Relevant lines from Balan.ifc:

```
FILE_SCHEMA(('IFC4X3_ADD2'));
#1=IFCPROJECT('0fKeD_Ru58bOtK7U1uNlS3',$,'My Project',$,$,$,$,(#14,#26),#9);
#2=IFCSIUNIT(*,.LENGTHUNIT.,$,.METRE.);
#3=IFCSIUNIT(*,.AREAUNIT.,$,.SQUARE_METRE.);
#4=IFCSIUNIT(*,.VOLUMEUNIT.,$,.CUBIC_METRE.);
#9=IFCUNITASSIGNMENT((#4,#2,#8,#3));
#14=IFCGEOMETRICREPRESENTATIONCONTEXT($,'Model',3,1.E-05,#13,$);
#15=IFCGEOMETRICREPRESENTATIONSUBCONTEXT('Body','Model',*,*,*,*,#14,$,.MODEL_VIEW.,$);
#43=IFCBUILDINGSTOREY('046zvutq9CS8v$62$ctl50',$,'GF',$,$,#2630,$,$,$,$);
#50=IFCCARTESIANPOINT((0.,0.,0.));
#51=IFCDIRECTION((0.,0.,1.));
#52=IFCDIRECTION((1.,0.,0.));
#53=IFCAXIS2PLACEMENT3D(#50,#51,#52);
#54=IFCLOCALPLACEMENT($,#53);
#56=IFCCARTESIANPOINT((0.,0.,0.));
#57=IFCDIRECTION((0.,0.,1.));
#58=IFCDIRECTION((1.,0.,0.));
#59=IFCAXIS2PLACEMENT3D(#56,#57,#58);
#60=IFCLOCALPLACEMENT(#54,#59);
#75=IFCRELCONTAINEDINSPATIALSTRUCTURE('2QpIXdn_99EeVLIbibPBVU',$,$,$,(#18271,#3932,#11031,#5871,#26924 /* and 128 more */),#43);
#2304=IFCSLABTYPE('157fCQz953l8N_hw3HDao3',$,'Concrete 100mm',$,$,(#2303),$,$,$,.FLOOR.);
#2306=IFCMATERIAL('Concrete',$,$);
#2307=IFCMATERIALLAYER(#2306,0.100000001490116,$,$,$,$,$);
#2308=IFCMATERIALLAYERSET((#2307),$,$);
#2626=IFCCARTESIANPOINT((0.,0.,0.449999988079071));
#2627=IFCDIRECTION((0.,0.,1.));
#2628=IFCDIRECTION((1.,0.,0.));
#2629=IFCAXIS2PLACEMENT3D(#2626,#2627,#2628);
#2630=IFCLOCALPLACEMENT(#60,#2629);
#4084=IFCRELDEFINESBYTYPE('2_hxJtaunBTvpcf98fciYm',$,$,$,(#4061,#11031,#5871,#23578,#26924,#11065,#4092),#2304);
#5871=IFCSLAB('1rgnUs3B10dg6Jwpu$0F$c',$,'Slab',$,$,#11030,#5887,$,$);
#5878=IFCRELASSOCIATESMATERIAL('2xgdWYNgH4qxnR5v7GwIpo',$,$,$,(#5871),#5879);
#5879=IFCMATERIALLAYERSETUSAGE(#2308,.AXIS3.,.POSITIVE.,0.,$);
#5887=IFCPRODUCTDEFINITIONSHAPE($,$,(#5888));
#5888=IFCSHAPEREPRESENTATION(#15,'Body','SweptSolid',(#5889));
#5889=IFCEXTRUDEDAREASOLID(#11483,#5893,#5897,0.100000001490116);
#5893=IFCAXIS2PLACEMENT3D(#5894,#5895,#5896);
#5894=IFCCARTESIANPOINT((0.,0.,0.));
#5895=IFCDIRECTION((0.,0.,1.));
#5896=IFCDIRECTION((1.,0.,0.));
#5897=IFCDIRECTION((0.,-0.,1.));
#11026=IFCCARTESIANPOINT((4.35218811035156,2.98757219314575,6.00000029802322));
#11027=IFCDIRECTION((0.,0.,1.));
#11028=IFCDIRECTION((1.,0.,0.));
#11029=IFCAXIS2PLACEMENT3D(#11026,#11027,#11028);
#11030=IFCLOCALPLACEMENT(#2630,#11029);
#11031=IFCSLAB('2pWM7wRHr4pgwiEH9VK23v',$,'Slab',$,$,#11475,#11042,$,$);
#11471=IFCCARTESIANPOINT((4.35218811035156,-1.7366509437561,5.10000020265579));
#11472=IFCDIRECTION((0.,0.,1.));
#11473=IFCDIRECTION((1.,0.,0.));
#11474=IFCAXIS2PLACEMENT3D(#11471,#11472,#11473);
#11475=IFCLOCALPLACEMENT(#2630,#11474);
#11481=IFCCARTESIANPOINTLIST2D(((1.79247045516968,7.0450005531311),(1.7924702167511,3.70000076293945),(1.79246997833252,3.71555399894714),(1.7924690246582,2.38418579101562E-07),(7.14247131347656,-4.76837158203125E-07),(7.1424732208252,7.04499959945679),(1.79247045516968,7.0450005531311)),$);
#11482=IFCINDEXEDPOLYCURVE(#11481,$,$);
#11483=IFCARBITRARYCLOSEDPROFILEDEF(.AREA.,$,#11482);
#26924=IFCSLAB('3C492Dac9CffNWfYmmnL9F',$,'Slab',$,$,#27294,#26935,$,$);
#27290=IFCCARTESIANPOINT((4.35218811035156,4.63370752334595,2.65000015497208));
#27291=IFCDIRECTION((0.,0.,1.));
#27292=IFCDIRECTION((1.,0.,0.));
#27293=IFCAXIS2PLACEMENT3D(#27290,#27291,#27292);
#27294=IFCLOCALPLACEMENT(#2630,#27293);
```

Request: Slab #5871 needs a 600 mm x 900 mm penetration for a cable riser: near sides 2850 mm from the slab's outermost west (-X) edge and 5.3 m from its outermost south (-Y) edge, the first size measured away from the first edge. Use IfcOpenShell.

```python
import numpy as np
import ifcopenshell
import ifcopenshell.api.feature
import ifcopenshell.api.geometry
import ifcopenshell.api.root
import ifcopenshell.geom
import ifcopenshell.util.placement
import ifcopenshell.util.representation
import ifcopenshell.util.shape
import ifcopenshell.util.unit

model = ifcopenshell.open("Balan.ifc")
unit_scale = ifcopenshell.util.unit.calculate_unit_scale(model)
settings = ifcopenshell.geom.settings()


def volume(element):
    """Net volume in cubic metres, openings subtracted."""
    shape = ifcopenshell.geom.create_shape(settings, element)
    return ifcopenshell.util.shape.get_volume(shape.geometry)


slab = model.by_guid("1rgnUs3B10dg6Jwpu$0F$c")
before = volume(slab)

# Extent in the slab's own axes, in metres. The edges named are its -X and -Y sides.
slab_shape = ifcopenshell.geom.create_shape(settings, slab)
vertices = ifcopenshell.util.shape.get_vertices(slab_shape.geometry)
x_min, y_min, bottom = vertices.min(axis=0)
top = vertices[:, 2].max()

opening = ifcopenshell.api.root.create_entity(model, ifc_class="IfcOpeningElement", name="Cable riser opening", predefined_type="OPENING")
context = ifcopenshell.util.representation.get_context(model, "Model", "Body", "MODEL_VIEW")
width, depth = 0.6, 0.9
outline = [(0.0, 0.0), (width, 0.0), (width, depth), (0.0, depth), (0.0, 0.0)]
# Overshoot both faces by 50 mm so the cut is clean.
shape = ifcopenshell.api.geometry.add_slab_representation(
    model, context=context, depth=top - bottom + 0.1, polyline=outline
)
ifcopenshell.api.geometry.assign_representation(model, product=opening, representation=shape)

matrix = ifcopenshell.util.placement.get_local_placement(slab.ObjectPlacement)
matrix[:, 3] = matrix @ np.append(np.array([x_min + 2.85, y_min + 5.3, bottom - 0.05]) / unit_scale, 1.0)
ifcopenshell.api.geometry.edit_object_placement(model, product=opening, matrix=matrix, is_si=False)
ifcopenshell.api.feature.add_feature(model, feature=opening, element=slab)

after = volume(slab)

print(f"slab volume {before:.3f} -> {after:.3f} m3")

model.write("Balan-out.ifc")
```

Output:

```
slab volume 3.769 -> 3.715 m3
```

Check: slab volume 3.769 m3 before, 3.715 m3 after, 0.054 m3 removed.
